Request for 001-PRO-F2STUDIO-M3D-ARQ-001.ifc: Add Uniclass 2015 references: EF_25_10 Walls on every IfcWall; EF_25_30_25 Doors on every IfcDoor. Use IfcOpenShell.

First a look at what the model holds.

```python
import ifcopenshell

model = ifcopenshell.open("001-PRO-F2STUDIO-M3D-ARQ-001.ifc")
print(model.schema)
print("classifications:", [c.Name for c in model.by_type("IfcClassification")])
for ifc_class in ("IfcDoor", "IfcRoof", "IfcStair", "IfcWall", "IfcWindow"):
    print(ifc_class, len(model.by_type(ifc_class)))
```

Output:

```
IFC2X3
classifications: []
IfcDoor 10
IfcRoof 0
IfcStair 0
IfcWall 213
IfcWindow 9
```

```python
import ifcopenshell
import ifcopenshell.api.classification

model = ifcopenshell.open("001-PRO-F2STUDIO-M3D-ARQ-001.ifc")

# IFC2X3 requires Source and Edition and has no link from the project to the system.
system = model.create_entity("IfcClassification", Source="NBS", Edition="2015", Name="Uniclass 2015")

codes = {
    "IfcWall": ("EF_25_10", "Walls"),
    "IfcDoor": ("EF_25_30_25", "Doors"),
}
for ifc_class, (code, name) in codes.items():
    products = model.by_type(ifc_class)
    ifcopenshell.api.classification.add_reference(
        model, products=products, classification=system, identification=code, name=name
    )
    print(code, len(products))

model.write("001-PRO-F2STUDIO-M3D-ARQ-001_rev.ifc")
```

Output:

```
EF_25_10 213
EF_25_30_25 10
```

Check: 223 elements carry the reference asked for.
